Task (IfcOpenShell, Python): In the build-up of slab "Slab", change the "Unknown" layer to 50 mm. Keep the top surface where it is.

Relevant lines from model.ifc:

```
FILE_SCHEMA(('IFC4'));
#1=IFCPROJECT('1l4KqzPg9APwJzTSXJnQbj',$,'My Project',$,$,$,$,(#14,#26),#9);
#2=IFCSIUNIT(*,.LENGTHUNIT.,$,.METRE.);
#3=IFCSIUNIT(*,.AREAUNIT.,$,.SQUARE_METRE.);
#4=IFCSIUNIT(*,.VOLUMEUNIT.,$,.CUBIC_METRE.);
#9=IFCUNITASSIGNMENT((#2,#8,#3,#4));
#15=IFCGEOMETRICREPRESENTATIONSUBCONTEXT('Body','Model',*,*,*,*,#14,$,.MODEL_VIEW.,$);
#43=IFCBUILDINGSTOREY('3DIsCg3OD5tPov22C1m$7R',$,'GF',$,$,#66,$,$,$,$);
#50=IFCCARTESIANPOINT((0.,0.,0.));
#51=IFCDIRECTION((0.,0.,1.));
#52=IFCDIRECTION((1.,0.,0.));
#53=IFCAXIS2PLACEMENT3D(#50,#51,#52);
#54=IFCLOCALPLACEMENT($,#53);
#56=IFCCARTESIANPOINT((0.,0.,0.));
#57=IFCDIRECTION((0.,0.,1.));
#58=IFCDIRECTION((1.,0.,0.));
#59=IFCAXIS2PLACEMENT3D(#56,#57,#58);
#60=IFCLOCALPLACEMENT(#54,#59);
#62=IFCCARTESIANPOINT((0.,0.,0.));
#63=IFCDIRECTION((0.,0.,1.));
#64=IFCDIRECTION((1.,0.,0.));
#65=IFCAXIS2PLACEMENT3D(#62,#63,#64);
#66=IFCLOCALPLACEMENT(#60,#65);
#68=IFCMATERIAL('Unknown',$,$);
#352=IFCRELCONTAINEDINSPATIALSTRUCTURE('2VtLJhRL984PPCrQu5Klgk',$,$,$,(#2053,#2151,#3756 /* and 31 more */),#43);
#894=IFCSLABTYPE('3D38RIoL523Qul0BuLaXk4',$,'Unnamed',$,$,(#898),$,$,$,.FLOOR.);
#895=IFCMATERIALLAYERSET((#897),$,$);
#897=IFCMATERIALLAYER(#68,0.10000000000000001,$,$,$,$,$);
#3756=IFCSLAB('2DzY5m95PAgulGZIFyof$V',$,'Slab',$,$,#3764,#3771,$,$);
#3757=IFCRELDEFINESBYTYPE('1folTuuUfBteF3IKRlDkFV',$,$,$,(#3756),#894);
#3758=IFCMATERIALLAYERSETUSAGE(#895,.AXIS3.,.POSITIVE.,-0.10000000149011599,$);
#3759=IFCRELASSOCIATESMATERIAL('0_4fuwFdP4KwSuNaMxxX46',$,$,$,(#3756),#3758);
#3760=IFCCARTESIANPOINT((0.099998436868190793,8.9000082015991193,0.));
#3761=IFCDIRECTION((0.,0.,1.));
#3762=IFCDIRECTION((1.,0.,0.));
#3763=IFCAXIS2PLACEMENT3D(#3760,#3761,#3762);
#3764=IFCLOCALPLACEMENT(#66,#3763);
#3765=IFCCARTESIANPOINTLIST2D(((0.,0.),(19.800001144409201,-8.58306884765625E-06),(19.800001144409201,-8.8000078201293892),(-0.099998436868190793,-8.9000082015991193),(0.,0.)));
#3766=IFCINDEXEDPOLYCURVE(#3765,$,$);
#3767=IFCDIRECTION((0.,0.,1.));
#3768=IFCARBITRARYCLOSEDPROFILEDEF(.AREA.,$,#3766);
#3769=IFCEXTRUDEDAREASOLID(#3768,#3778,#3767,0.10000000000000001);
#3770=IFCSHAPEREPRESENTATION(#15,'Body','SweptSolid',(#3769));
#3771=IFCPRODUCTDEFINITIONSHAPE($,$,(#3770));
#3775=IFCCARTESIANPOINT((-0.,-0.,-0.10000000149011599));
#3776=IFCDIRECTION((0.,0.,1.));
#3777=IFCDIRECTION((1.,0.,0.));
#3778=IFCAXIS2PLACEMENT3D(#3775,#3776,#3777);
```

```python
import ifcopenshell
import ifcopenshell.util.element
import ifcopenshell.util.representation
import ifcopenshell.util.unit

model = ifcopenshell.open("model.ifc")
unit_scale = ifcopenshell.util.unit.calculate_unit_scale(model)

layer_set = model.by_id(895)
layer = next(l for l in layer_set.MaterialLayers if l.Material and l.Material.Name == "Unknown")
change = 0.05 / unit_scale - layer.LayerThickness
layer.LayerThickness += change

# Geometry does not follow the layer set by itself.
slabs = [e for e in ifcopenshell.util.element.get_elements_by_material(model, layer_set) if e.is_a("IfcSlab")]
for slab in sorted(slabs, key=lambda e: e.id()):
    body = ifcopenshell.util.representation.get_representation(slab, "Model", "Body")
    solid = body.Items[0]
    old_depth = solid.Depth
    solid.Depth += change
    # Extruded upwards: lower the start of the extrusion so the top stays.
    x, y, z = solid.Position.Location.Coordinates
    solid.Position.Location = model.createIfcCartesianPoint((x, y, z - change))
    print(slab.id(), f"{old_depth:g} -> {solid.Depth:g}")

# The layers are counted up from the underside, which has moved.
for usage in {ifcopenshell.util.element.get_material(slab) for slab in slabs}:
    usage.OffsetFromReferenceLine -= change

model.write("model-out.ifc")
```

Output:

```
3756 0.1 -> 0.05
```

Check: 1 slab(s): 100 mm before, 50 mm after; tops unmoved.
